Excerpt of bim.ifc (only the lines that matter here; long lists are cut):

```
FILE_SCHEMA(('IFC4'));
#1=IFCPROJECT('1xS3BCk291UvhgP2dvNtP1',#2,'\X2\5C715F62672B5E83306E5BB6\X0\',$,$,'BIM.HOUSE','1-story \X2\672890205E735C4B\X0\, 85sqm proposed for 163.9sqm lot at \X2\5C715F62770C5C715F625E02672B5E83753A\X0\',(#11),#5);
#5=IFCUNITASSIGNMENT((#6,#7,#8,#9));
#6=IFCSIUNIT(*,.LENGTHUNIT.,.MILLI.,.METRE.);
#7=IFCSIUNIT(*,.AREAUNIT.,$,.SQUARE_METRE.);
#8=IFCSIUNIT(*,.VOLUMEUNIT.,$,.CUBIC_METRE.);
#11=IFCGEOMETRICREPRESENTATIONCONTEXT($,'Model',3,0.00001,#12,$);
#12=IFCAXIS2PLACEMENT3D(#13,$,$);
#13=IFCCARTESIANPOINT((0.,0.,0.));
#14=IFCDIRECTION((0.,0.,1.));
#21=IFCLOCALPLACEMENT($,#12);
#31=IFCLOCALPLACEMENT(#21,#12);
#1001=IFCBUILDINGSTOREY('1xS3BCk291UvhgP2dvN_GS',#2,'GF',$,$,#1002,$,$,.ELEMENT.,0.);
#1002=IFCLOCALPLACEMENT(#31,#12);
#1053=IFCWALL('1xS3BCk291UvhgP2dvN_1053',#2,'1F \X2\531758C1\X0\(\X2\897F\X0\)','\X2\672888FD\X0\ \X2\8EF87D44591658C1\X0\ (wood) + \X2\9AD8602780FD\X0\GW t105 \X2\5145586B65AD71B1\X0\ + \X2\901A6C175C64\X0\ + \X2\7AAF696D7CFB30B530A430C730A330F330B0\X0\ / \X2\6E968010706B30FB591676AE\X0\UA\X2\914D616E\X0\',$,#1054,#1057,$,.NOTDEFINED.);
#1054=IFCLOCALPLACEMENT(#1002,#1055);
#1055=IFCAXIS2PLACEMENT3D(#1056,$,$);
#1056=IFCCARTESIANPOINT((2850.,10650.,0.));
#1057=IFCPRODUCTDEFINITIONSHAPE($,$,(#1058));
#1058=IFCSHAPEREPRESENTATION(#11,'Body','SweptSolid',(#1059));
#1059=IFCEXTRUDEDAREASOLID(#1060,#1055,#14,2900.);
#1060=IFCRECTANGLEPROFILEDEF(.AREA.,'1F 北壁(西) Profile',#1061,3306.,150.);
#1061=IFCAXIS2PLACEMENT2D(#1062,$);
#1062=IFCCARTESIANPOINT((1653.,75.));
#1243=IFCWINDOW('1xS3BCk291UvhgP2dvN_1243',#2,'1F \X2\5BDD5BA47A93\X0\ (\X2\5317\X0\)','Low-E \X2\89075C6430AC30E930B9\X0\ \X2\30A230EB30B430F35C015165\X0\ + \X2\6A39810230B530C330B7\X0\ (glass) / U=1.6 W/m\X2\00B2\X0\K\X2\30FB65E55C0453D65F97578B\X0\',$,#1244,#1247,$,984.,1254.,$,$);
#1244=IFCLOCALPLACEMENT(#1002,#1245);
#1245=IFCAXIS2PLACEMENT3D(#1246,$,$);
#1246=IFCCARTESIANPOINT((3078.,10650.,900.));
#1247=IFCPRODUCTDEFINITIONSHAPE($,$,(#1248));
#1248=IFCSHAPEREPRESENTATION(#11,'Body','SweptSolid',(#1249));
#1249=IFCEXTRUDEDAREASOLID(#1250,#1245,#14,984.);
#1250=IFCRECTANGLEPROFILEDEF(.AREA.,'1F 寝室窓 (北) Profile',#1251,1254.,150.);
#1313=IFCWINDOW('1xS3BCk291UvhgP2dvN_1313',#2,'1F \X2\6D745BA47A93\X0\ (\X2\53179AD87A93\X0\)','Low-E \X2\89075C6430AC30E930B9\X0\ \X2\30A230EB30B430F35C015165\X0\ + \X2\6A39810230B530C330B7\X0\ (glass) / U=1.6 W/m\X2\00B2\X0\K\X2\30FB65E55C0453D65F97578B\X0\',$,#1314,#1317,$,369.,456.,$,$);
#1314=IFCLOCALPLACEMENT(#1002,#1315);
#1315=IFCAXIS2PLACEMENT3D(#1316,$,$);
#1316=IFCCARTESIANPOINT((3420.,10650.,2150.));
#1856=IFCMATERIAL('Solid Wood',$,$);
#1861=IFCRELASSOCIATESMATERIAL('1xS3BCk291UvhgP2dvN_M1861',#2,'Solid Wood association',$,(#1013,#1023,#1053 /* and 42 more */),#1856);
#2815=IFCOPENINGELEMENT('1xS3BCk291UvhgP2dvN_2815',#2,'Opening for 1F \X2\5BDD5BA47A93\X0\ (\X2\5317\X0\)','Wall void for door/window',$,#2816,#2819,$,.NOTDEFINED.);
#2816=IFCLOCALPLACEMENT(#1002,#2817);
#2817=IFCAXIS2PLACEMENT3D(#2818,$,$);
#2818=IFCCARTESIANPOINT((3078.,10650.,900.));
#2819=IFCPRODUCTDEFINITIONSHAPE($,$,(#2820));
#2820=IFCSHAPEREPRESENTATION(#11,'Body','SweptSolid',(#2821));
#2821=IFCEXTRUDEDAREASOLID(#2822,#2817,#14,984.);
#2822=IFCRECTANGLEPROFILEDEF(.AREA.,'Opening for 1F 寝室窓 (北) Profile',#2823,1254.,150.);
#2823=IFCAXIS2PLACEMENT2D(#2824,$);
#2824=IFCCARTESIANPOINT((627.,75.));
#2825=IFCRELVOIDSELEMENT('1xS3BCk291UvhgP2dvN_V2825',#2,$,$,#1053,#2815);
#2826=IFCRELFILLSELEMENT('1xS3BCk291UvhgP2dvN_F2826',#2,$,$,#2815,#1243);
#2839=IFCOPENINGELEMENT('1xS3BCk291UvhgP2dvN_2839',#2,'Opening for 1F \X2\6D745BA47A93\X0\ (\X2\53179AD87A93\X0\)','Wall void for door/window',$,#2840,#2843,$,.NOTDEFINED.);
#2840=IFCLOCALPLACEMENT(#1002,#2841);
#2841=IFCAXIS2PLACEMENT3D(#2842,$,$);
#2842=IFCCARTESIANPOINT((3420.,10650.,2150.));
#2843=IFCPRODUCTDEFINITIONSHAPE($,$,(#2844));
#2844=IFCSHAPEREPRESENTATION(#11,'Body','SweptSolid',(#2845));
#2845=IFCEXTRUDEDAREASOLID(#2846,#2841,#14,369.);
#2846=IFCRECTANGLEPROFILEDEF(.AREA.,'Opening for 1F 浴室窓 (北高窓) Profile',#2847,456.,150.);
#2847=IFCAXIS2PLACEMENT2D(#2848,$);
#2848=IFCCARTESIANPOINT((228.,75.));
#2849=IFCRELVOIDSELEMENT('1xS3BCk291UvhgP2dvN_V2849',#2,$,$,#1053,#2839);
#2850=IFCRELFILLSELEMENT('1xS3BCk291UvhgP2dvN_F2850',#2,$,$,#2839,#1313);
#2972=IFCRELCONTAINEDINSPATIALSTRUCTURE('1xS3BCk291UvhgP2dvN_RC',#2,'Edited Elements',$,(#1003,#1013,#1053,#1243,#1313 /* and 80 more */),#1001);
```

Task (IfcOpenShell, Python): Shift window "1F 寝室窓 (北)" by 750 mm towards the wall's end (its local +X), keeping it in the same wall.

```python
import ifcopenshell
import ifcopenshell.api.geometry
import ifcopenshell.util.placement

model = ifcopenshell.open("bim.ifc")

window = model.by_guid("1xS3BCk291UvhgP2dvN_1243")
opening = window.FillsVoids[0].RelatingOpeningElement
wall = opening.VoidsElements[0].RelatingBuildingElement

wall_matrix = ifcopenshell.util.placement.get_local_placement(wall.ObjectPlacement)
shift = wall_matrix[:3, 0] * 750.0
before = ifcopenshell.util.placement.get_local_placement(window.ObjectPlacement)[:3, 3].copy()

# The window is not placed relative to its opening, so move both.
for product in (opening, window):
    matrix = ifcopenshell.util.placement.get_local_placement(product.ObjectPlacement)
    matrix[:3, 3] += shift
    ifcopenshell.api.geometry.edit_object_placement(model, product=product, matrix=matrix, is_si=False)

after = ifcopenshell.util.placement.get_local_placement(window.ObjectPlacement)[:3, 3]
print("window moved by", (after - before).round(3) + 0.0)

model.write("bim_edited.ifc")
```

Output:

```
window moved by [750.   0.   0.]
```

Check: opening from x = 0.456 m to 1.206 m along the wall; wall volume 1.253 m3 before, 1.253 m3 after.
